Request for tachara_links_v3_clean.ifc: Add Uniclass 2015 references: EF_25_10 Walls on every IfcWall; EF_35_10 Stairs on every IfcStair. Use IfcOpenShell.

First a look at what the model holds.

```python
import ifcopenshell

model = ifcopenshell.open("tachara_links_v3_clean.ifc")
print(model.schema)
print("classifications:", [c.Name for c in model.by_type("IfcClassification")])
for ifc_class in ("IfcDoor", "IfcRoof", "IfcStair", "IfcWall", "IfcWindow"):
    print(ifc_class, len(model.by_type(ifc_class)))
```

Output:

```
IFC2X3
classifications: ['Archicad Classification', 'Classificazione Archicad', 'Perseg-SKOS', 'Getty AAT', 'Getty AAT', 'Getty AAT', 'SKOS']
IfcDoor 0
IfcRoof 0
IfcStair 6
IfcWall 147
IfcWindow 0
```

```python
import ifcopenshell
import ifcopenshell.api.classification

model = ifcopenshell.open("tachara_links_v3_clean.ifc")

# IFC2X3 requires Source and Edition and has no link from the project to the system.
system = model.create_entity("IfcClassification", Source="NBS", Edition="2015", Name="Uniclass 2015")

codes = {
    "IfcWall": ("EF_25_10", "Walls"),
    "IfcStair": ("EF_35_10", "Stairs"),
}
for ifc_class, (code, name) in codes.items():
    products = model.by_type(ifc_class)
    ifcopenshell.api.classification.add_reference(
        model, products=products, classification=system, identification=code, name=name
    )
    print(code, len(products))

model.write("tachara_links_v3_clean_v2.ifc")
```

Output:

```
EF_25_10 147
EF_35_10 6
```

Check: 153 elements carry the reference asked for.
